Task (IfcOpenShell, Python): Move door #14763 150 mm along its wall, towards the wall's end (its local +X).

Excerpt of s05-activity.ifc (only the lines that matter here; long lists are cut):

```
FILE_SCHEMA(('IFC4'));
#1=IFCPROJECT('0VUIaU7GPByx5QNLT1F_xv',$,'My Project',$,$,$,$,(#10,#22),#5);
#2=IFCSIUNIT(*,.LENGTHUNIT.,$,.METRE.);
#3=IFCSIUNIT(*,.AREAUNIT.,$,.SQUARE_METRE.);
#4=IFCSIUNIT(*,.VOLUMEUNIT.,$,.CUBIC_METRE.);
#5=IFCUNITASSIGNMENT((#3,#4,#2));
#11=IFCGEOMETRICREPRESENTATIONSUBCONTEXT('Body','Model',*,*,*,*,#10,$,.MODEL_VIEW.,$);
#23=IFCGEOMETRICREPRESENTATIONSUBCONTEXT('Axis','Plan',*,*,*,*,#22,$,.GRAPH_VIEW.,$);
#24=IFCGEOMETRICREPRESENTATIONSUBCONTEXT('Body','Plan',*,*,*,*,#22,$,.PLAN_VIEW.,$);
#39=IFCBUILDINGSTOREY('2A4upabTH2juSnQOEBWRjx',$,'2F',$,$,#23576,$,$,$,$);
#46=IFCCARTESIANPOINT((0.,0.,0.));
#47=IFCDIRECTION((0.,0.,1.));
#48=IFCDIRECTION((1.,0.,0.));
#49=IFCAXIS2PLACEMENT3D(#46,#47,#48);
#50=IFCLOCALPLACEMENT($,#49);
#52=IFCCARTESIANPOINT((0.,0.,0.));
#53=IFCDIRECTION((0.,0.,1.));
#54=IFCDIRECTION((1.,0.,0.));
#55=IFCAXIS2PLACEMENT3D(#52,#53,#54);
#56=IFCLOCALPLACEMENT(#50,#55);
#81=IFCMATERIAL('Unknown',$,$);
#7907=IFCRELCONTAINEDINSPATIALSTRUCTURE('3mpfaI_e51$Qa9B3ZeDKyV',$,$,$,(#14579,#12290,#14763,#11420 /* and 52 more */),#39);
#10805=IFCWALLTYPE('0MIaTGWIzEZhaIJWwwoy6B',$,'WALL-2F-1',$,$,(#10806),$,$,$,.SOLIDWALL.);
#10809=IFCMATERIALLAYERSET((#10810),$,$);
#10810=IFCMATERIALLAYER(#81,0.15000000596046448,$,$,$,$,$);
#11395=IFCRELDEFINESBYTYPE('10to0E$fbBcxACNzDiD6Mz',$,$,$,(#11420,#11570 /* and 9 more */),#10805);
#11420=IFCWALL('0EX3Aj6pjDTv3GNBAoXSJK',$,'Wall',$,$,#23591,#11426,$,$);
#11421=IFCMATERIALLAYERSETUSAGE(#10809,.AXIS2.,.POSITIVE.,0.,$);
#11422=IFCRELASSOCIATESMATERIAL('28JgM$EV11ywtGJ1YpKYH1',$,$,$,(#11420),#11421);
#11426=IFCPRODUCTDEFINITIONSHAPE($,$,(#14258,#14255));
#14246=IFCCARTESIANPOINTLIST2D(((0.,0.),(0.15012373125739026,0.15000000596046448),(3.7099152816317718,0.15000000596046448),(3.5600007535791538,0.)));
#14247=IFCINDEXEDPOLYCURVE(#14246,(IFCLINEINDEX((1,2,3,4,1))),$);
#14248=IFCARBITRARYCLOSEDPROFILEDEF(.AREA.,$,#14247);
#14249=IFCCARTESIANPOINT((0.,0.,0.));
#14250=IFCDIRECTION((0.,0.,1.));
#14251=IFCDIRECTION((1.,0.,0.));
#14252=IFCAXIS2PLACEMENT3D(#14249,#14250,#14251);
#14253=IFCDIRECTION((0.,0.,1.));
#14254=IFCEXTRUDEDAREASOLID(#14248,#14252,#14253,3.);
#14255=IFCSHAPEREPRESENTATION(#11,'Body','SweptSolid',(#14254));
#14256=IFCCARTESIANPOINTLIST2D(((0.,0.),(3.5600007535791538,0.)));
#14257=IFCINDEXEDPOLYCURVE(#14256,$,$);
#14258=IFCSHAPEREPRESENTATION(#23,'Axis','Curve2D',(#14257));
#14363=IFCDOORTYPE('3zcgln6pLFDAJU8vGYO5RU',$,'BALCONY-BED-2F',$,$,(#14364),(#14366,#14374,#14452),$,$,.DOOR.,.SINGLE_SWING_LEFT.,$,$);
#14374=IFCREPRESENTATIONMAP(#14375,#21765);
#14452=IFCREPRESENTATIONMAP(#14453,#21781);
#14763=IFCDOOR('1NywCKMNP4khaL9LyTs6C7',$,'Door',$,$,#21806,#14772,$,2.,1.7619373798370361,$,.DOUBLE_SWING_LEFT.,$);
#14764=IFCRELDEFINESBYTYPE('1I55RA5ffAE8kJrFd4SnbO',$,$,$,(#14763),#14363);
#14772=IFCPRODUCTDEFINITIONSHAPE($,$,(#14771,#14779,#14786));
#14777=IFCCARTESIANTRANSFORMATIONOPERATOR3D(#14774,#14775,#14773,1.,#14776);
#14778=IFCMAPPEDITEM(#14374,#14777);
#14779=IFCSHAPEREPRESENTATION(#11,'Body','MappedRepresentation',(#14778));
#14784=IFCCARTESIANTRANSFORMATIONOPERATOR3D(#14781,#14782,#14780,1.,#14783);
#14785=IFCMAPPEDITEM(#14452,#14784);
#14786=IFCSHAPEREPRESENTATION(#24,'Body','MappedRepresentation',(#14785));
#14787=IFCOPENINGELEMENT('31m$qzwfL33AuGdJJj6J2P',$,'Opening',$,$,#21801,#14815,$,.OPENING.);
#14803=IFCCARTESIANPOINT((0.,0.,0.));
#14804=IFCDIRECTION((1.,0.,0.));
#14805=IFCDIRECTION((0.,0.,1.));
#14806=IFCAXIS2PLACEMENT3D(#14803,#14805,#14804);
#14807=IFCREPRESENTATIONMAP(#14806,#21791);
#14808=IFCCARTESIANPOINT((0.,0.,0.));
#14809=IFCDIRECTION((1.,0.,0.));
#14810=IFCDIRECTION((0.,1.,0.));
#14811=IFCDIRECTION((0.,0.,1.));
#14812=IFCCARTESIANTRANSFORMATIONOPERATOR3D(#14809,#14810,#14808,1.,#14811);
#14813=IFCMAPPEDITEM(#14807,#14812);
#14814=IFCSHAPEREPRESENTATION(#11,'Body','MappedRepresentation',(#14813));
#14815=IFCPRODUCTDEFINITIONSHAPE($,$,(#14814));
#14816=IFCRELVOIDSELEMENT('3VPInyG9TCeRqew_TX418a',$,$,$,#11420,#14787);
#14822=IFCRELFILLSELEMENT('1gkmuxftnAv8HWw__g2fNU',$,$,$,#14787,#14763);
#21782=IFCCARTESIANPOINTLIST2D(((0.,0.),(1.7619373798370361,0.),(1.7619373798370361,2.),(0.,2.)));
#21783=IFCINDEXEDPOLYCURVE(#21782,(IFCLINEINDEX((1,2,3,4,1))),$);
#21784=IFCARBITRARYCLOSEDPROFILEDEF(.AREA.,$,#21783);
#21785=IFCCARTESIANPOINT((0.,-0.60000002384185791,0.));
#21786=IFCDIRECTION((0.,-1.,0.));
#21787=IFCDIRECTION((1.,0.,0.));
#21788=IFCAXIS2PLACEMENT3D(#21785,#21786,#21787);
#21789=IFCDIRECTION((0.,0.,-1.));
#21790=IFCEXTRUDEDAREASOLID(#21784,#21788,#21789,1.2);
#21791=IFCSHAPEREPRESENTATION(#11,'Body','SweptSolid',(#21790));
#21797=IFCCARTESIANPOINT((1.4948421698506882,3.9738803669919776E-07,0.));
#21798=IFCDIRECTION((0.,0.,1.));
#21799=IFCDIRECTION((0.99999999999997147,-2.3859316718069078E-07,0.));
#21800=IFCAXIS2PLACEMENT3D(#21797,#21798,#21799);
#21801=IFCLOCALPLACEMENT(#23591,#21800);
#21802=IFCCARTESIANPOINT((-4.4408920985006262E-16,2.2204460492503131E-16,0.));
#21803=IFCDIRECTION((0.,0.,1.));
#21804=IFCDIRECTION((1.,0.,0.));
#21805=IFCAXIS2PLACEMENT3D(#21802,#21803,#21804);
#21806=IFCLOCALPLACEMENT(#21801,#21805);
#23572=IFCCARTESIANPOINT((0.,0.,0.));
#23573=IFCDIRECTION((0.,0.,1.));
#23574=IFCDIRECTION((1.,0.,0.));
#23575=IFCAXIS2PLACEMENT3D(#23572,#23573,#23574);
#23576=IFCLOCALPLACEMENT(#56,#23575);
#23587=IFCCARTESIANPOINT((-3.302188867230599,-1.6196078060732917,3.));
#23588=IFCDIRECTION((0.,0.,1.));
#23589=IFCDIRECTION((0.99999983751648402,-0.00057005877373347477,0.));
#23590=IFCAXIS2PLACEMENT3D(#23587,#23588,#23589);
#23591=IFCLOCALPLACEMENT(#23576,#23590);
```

```python
import ifcopenshell
import ifcopenshell.api.geometry
import ifcopenshell.util.placement
import ifcopenshell.util.unit

model = ifcopenshell.open("s05-activity.ifc")
unit_scale = ifcopenshell.util.unit.calculate_unit_scale(model)

door = model.by_guid("1NywCKMNP4khaL9LyTs6C7")
opening = door.FillsVoids[0].RelatingOpeningElement
wall = opening.VoidsElements[0].RelatingBuildingElement

wall_matrix = ifcopenshell.util.placement.get_local_placement(wall.ObjectPlacement)
shift = wall_matrix[:3, 0] * 0.15 / unit_scale
before = ifcopenshell.util.placement.get_local_placement(door.ObjectPlacement)[:3, 3].copy()

# The door is placed relative to its opening, so it follows when the opening moves.
matrix = ifcopenshell.util.placement.get_local_placement(opening.ObjectPlacement)
matrix[:3, 3] += shift
ifcopenshell.api.geometry.edit_object_placement(
    model, product=opening, matrix=matrix, is_si=False, should_transform_children=True
)

after = ifcopenshell.util.placement.get_local_placement(door.ObjectPlacement)[:3, 3]
print("door moved by", (after - before).round(3) + 0.0)

model.write("s05-activity-out.ifc")
```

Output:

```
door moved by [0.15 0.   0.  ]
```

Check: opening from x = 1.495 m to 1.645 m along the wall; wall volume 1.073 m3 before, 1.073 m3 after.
